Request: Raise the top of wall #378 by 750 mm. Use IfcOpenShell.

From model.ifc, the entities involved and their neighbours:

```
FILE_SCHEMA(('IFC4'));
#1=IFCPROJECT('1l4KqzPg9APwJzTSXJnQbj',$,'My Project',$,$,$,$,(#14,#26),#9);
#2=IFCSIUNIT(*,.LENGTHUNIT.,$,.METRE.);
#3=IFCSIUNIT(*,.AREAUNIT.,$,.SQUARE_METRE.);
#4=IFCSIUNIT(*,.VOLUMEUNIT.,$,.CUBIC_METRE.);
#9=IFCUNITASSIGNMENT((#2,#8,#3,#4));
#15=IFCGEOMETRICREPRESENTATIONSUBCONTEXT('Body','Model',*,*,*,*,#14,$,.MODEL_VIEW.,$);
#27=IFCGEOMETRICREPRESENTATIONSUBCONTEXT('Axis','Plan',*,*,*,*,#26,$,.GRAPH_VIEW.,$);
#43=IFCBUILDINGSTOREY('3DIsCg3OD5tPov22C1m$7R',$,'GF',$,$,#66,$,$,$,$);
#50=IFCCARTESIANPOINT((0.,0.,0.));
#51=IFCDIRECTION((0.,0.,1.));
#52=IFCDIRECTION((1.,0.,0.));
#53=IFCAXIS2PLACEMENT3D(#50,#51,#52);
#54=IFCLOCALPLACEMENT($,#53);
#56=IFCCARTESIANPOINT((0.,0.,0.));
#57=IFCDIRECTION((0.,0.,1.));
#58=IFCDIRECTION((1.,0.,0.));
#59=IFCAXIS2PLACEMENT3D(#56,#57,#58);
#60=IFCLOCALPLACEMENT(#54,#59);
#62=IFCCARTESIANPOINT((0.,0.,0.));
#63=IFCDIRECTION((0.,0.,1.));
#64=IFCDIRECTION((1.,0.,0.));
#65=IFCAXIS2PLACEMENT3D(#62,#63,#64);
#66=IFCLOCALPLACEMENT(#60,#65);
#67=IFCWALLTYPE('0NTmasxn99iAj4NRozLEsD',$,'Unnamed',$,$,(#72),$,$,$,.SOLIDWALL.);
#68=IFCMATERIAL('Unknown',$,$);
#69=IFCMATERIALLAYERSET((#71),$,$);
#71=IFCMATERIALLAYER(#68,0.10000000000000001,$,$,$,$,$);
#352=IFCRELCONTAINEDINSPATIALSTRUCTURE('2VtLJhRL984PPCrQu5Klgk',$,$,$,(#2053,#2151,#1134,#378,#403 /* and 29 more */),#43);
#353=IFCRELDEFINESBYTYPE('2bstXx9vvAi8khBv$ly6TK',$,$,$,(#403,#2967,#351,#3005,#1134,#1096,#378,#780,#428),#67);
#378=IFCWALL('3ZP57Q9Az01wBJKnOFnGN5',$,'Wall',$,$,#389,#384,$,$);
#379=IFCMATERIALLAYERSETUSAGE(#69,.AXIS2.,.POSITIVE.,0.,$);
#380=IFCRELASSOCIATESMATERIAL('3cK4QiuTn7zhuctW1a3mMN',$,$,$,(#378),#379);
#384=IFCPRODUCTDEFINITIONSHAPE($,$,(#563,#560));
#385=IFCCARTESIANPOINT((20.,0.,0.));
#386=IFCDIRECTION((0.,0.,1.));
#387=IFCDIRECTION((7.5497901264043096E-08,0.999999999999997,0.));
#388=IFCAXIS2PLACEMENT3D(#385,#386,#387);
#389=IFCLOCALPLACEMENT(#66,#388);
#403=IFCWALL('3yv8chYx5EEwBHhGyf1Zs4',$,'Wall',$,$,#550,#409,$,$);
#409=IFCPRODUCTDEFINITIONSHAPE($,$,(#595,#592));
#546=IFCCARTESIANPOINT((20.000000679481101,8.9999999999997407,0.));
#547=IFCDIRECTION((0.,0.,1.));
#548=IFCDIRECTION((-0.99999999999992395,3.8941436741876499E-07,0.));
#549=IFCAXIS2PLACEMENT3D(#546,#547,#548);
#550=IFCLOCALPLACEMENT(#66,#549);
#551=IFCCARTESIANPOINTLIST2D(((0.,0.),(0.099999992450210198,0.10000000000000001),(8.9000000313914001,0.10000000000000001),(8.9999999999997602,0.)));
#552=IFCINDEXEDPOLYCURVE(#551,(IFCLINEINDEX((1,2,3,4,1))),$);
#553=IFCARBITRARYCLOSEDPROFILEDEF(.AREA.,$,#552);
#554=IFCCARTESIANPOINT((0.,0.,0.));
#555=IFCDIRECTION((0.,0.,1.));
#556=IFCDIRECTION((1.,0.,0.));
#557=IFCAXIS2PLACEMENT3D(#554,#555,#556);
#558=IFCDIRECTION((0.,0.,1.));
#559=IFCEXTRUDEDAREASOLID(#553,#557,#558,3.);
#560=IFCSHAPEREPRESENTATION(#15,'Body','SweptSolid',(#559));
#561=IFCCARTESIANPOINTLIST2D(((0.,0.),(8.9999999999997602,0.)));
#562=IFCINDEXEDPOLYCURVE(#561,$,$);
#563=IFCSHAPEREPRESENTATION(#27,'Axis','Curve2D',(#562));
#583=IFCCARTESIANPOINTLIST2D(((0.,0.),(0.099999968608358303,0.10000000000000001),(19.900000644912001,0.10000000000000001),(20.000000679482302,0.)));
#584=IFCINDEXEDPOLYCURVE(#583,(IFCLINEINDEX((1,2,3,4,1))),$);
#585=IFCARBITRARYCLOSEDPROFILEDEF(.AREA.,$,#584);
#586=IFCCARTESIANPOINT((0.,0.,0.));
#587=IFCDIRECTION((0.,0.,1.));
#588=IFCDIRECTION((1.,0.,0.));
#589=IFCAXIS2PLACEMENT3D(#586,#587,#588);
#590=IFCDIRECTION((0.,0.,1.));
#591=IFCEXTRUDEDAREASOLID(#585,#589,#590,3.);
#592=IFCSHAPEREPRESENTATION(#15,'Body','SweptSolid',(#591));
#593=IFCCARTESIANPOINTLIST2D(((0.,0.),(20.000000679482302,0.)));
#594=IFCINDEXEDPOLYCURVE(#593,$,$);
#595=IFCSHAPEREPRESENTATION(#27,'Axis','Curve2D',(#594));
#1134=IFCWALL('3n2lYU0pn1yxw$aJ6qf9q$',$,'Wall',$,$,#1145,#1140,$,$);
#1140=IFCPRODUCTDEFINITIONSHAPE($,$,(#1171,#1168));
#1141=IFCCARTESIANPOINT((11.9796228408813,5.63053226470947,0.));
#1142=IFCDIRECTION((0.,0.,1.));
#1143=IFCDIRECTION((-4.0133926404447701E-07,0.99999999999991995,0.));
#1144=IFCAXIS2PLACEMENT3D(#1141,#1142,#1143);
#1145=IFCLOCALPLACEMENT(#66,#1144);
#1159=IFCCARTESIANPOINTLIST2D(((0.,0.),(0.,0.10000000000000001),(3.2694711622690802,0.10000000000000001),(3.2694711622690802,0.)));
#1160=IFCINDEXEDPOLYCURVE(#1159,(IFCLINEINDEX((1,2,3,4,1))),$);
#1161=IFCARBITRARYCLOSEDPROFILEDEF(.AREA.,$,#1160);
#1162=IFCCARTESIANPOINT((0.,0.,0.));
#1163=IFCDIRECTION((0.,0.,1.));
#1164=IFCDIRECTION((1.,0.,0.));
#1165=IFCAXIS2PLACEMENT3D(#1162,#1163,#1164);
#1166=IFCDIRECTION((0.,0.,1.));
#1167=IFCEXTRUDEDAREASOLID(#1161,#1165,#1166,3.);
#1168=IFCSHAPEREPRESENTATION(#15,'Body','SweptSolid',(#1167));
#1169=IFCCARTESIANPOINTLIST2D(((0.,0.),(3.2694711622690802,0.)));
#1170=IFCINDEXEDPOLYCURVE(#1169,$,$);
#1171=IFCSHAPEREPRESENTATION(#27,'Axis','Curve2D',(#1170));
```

```python
import ifcopenshell
import ifcopenshell.geom
import ifcopenshell.util.representation
import ifcopenshell.util.shape
import ifcopenshell.util.unit

model = ifcopenshell.open("model.ifc")
unit_scale = ifcopenshell.util.unit.calculate_unit_scale(model)
settings = ifcopenshell.geom.settings()


def volume(element):
    """Net volume in cubic metres, openings subtracted."""
    shape = ifcopenshell.geom.create_shape(settings, element)
    return ifcopenshell.util.shape.get_volume(shape.geometry)


wall = model.by_guid("3ZP57Q9Az01wBJKnOFnGN5")
before = volume(wall)

body = ifcopenshell.util.representation.get_representation(wall, "Model", "Body")
solid = body.Items[0]
old_height = solid.Depth
solid.Depth += 0.75 / unit_scale
after = volume(wall)

print(f"height {old_height:g} -> {solid.Depth:g}, volume {before:.3f} -> {after:.3f} m3")

model.write("model-out.ifc")
```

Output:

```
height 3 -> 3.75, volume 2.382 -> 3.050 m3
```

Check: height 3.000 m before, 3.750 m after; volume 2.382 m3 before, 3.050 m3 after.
